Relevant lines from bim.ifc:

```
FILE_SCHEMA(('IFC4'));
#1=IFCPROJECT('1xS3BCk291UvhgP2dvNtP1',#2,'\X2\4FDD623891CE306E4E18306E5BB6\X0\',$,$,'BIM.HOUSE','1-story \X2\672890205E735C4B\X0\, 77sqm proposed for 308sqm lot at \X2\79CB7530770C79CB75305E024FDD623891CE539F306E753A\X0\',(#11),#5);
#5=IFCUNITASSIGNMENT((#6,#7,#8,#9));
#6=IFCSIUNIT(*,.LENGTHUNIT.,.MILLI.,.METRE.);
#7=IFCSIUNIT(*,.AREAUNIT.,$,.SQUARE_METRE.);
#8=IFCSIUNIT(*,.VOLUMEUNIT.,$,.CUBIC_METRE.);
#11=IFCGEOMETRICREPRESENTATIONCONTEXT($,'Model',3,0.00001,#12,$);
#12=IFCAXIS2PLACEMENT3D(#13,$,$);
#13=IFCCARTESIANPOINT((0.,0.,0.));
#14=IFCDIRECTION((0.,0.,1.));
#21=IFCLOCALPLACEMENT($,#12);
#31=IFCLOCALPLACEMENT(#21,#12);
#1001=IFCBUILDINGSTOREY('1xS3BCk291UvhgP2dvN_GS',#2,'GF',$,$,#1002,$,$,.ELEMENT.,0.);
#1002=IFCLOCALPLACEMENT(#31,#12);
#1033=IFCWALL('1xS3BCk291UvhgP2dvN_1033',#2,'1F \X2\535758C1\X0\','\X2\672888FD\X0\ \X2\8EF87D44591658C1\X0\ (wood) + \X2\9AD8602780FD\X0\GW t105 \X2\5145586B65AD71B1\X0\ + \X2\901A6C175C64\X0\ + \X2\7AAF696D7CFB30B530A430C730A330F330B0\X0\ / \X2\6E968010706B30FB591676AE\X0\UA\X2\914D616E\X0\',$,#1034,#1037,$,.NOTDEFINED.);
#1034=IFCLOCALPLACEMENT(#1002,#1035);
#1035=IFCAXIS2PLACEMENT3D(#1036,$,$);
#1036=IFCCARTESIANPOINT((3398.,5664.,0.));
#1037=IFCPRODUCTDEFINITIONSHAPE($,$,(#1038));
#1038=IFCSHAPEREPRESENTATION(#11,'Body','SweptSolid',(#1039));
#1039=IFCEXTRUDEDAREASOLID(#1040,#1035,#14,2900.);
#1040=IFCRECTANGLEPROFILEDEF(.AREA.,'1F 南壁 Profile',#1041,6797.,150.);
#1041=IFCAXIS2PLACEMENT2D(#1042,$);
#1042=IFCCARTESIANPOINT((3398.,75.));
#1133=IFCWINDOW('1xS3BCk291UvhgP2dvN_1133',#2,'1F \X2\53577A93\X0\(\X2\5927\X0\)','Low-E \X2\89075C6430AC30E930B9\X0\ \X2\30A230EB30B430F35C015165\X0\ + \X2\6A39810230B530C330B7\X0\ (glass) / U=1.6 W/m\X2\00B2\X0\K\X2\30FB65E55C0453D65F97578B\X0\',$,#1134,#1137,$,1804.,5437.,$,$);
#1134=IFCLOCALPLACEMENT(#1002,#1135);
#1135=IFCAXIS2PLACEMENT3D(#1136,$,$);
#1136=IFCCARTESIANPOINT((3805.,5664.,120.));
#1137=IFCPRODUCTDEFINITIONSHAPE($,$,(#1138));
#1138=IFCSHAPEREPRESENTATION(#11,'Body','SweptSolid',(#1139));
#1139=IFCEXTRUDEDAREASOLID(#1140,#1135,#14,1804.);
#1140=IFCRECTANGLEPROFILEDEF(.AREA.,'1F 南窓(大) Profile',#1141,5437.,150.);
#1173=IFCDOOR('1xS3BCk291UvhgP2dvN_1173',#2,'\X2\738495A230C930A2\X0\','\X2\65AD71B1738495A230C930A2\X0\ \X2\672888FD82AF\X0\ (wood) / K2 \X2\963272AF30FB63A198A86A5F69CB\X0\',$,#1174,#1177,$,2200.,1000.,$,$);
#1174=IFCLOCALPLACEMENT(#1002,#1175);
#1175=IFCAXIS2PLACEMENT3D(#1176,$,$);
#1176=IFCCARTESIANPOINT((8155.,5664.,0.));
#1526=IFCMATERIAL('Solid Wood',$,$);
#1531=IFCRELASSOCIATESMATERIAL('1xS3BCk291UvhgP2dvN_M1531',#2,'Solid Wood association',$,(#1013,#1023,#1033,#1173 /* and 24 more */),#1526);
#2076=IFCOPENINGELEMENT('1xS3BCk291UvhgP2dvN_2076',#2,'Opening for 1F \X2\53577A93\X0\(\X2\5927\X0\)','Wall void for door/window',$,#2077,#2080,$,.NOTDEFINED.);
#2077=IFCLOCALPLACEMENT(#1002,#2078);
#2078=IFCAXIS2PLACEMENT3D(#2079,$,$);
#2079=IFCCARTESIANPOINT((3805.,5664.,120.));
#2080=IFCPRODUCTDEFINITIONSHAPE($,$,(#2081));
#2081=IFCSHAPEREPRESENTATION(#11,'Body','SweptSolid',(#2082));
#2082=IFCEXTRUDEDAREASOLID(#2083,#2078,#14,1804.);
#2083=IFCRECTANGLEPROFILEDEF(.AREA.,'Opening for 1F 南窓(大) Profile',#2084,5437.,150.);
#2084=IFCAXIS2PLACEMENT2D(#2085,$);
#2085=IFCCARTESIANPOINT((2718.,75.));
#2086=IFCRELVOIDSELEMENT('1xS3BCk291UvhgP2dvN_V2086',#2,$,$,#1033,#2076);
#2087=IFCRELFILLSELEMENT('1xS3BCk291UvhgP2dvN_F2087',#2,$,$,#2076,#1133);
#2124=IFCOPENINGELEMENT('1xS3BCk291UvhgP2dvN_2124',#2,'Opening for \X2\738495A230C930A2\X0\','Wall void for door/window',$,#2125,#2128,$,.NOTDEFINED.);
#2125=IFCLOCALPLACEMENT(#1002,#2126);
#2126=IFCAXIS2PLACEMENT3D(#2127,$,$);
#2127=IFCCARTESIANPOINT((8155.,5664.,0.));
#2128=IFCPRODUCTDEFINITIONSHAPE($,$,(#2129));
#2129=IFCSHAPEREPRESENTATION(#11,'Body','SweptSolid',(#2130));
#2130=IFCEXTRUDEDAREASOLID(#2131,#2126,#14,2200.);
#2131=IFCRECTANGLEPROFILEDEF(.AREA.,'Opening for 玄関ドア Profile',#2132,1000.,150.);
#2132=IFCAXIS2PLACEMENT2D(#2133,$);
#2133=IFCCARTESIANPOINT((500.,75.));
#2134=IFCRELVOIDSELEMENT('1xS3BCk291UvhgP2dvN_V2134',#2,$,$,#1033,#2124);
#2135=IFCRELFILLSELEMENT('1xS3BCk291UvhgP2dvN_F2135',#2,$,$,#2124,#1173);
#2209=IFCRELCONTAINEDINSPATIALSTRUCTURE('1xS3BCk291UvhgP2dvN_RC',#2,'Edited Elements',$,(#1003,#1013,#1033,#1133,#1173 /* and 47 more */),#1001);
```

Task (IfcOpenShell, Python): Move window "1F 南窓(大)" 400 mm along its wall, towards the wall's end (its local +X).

```python
import ifcopenshell
import ifcopenshell.api.geometry
import ifcopenshell.util.placement
import ifcopenshell.util.unit

model = ifcopenshell.open("bim.ifc")
unit_scale = ifcopenshell.util.unit.calculate_unit_scale(model)

window = model.by_guid("1xS3BCk291UvhgP2dvN_1133")
opening = window.FillsVoids[0].RelatingOpeningElement
wall = opening.VoidsElements[0].RelatingBuildingElement

wall_matrix = ifcopenshell.util.placement.get_local_placement(wall.ObjectPlacement)
shift = wall_matrix[:3, 0] * 0.4 / unit_scale
before = ifcopenshell.util.placement.get_local_placement(window.ObjectPlacement)[:3, 3].copy()

# The window is not placed relative to its opening, so move both.
for product in (opening, window):
    matrix = ifcopenshell.util.placement.get_local_placement(product.ObjectPlacement)
    matrix[:3, 3] += shift
    ifcopenshell.api.geometry.edit_object_placement(model, product=product, matrix=matrix, is_si=False)

after = ifcopenshell.util.placement.get_local_placement(window.ObjectPlacement)[:3, 3]
print("window moved by", (after - before).round(3) + 0.0)

model.write("bim_rev.ifc")
```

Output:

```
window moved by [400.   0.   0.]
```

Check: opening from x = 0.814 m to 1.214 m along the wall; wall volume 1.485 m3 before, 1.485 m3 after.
